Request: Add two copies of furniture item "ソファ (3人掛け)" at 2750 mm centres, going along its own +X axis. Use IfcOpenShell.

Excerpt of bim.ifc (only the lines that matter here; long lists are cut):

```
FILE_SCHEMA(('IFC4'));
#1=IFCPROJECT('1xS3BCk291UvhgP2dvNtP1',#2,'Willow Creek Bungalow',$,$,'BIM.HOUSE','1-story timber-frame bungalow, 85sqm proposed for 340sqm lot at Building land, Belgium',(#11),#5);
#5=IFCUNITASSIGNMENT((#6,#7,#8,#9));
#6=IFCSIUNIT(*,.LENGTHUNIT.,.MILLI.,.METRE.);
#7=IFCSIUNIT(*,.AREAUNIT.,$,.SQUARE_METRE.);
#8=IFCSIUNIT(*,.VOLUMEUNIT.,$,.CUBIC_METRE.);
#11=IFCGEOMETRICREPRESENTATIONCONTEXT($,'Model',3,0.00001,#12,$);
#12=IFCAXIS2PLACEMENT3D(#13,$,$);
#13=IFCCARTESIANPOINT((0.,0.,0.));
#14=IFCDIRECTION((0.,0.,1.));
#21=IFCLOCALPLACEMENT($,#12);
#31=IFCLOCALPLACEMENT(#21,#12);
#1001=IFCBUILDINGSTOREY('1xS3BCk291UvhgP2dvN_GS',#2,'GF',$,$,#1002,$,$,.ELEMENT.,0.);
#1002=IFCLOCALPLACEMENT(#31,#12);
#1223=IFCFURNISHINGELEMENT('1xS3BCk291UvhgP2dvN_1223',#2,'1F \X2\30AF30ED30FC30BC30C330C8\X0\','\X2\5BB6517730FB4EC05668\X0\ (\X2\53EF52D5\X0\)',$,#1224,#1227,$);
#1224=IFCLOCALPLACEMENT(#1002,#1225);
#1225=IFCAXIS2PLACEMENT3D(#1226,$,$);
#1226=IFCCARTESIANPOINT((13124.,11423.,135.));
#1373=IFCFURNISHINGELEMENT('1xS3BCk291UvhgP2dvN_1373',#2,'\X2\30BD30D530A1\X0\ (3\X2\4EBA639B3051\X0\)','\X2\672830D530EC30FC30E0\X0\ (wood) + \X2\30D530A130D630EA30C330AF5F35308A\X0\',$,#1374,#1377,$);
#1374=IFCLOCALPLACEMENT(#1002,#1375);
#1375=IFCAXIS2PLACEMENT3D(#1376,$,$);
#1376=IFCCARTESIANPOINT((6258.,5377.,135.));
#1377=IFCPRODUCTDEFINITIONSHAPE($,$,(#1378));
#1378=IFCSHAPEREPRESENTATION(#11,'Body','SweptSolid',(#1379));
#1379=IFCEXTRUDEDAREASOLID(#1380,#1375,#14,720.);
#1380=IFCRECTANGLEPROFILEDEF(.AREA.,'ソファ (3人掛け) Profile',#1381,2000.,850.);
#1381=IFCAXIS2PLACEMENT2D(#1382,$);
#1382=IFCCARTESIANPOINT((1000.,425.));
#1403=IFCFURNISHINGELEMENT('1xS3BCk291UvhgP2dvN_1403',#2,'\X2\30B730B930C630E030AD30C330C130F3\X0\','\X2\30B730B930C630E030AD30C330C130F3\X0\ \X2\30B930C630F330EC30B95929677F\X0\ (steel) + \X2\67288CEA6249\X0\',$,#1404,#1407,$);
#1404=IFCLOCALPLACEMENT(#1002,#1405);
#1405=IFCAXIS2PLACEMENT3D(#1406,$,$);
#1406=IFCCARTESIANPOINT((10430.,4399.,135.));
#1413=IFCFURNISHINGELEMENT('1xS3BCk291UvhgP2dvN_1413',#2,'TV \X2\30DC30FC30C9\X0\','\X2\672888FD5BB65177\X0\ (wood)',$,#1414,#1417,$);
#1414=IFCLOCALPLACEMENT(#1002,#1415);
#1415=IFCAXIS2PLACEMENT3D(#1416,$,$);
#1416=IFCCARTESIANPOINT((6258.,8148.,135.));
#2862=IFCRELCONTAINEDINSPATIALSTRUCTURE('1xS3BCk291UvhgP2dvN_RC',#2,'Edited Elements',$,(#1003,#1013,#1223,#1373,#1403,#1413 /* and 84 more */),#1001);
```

```python
import ifcopenshell
import ifcopenshell.api.geometry
import ifcopenshell.api.root
import ifcopenshell.util.element
import ifcopenshell.util.placement

model = ifcopenshell.open("bim.ifc")


def reuse_history(source, copy):
    """copy_class also copies each property set's owner history, people and application; keep the originals."""
    for rel in copy.IsDefinedBy:
        if rel.is_a("IfcRelDefinesByProperties") and (history := rel.RelatingPropertyDefinition.OwnerHistory):
            rel.RelatingPropertyDefinition.OwnerHistory = source.OwnerHistory
            ifcopenshell.util.element.remove_deep2(model, history)


source = model.by_id(1373)
base = ifcopenshell.util.placement.get_local_placement(source.ObjectPlacement)
step = base[:3, 0] * 2750.0

for i in range(1, 3):
    copy = ifcopenshell.api.root.copy_class(model, product=source)
    copy.Representation = ifcopenshell.util.element.copy_deep(
        model, source.Representation, exclude=["IfcGeometricRepresentationContext", "IfcRepresentationMap"]
    )
    reuse_history(source, copy)
    matrix = base.copy()
    matrix[:3, 3] += i * step
    print("added at", matrix[:3, 3].round(3) + 0.0)
    ifcopenshell.api.geometry.edit_object_placement(model, product=copy, matrix=matrix, is_si=False)

model.write("bim_rev.ifc")
```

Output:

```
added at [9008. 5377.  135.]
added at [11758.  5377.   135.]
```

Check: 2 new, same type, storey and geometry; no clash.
